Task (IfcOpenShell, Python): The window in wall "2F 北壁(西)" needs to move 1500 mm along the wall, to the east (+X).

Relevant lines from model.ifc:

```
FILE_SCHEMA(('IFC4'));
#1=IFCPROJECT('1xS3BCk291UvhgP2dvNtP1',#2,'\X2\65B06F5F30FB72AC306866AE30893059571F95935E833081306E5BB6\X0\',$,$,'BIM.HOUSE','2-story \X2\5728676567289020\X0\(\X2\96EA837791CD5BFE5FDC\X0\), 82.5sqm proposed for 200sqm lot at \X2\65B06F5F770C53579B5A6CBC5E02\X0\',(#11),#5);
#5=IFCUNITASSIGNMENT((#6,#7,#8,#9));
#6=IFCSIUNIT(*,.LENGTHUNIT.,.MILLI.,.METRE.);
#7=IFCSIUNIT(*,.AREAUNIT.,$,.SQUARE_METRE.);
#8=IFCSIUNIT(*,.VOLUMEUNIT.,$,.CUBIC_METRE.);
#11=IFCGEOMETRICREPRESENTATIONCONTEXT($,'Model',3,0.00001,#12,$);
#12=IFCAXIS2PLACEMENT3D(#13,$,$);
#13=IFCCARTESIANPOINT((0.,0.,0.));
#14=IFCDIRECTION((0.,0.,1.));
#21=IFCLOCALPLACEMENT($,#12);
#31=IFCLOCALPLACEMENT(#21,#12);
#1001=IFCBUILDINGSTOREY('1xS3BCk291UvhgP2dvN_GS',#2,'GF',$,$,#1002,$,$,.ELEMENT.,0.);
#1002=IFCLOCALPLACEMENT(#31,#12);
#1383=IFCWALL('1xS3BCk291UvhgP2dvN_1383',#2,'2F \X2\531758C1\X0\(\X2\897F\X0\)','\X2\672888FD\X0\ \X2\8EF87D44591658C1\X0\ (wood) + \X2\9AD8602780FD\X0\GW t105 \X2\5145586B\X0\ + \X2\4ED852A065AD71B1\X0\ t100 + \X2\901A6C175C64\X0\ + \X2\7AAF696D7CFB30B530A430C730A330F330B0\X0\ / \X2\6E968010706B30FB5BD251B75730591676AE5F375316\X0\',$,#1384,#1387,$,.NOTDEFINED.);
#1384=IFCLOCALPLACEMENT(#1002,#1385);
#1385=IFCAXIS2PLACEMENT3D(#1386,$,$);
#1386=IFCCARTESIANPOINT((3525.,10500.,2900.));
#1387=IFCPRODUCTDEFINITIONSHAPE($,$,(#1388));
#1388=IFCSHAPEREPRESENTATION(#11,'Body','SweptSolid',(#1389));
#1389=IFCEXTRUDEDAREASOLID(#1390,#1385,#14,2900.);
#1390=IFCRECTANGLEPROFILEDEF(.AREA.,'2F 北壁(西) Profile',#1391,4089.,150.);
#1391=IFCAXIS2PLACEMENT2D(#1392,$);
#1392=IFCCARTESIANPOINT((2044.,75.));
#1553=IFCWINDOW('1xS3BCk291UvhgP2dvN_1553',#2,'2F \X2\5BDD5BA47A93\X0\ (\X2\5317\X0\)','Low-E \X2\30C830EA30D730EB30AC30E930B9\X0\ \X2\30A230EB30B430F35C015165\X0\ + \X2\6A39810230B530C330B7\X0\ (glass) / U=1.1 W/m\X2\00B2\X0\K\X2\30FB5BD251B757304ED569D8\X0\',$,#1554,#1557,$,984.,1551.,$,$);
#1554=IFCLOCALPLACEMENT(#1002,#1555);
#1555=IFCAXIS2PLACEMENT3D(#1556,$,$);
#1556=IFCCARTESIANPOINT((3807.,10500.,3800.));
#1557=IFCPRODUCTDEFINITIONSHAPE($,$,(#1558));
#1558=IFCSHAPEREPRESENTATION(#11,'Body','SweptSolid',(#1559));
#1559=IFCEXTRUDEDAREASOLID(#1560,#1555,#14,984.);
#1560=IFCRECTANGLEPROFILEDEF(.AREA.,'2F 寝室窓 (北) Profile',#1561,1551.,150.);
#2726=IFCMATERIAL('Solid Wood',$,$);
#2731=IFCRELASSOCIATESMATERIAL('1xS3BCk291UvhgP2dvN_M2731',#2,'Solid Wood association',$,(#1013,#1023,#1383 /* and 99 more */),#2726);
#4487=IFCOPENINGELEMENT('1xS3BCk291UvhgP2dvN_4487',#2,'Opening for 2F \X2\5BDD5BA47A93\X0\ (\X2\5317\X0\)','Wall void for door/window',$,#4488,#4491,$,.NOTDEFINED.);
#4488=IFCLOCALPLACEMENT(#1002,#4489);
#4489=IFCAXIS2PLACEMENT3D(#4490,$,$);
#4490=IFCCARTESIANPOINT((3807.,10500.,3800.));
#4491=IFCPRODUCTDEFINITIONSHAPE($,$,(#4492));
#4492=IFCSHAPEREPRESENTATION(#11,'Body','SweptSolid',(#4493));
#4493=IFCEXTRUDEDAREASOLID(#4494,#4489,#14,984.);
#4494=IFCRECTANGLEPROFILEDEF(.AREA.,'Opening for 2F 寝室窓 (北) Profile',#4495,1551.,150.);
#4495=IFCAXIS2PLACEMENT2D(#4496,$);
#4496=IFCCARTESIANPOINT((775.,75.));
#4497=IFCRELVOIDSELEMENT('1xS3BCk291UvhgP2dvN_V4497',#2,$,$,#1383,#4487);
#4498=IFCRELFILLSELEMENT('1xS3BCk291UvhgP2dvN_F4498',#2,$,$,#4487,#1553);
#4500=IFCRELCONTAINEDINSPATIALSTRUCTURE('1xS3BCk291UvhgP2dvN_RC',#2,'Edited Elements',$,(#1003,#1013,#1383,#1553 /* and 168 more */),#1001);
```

```python
import ifcopenshell
import ifcopenshell.api.geometry
import ifcopenshell.util.placement
import ifcopenshell.util.unit

model = ifcopenshell.open("model.ifc")
unit_scale = ifcopenshell.util.unit.calculate_unit_scale(model)

window = model.by_id(1553)
opening = window.FillsVoids[0].RelatingOpeningElement
wall = opening.VoidsElements[0].RelatingBuildingElement

wall_matrix = ifcopenshell.util.placement.get_local_placement(wall.ObjectPlacement)
shift = wall_matrix[:3, 0] * 1.5 / unit_scale
before = ifcopenshell.util.placement.get_local_placement(window.ObjectPlacement)[:3, 3].copy()

# The window is not placed relative to its opening, so move both.
for product in (opening, window):
    matrix = ifcopenshell.util.placement.get_local_placement(product.ObjectPlacement)
    matrix[:3, 3] += shift
    ifcopenshell.api.geometry.edit_object_placement(model, product=product, matrix=matrix, is_si=False)

after = ifcopenshell.util.placement.get_local_placement(window.ObjectPlacement)[:3, 3]
print("window moved by", (after - before).round(3) + 0.0)

model.write("model-out.ifc")
```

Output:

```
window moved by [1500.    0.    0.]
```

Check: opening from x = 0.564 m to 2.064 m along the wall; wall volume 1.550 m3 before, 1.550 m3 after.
